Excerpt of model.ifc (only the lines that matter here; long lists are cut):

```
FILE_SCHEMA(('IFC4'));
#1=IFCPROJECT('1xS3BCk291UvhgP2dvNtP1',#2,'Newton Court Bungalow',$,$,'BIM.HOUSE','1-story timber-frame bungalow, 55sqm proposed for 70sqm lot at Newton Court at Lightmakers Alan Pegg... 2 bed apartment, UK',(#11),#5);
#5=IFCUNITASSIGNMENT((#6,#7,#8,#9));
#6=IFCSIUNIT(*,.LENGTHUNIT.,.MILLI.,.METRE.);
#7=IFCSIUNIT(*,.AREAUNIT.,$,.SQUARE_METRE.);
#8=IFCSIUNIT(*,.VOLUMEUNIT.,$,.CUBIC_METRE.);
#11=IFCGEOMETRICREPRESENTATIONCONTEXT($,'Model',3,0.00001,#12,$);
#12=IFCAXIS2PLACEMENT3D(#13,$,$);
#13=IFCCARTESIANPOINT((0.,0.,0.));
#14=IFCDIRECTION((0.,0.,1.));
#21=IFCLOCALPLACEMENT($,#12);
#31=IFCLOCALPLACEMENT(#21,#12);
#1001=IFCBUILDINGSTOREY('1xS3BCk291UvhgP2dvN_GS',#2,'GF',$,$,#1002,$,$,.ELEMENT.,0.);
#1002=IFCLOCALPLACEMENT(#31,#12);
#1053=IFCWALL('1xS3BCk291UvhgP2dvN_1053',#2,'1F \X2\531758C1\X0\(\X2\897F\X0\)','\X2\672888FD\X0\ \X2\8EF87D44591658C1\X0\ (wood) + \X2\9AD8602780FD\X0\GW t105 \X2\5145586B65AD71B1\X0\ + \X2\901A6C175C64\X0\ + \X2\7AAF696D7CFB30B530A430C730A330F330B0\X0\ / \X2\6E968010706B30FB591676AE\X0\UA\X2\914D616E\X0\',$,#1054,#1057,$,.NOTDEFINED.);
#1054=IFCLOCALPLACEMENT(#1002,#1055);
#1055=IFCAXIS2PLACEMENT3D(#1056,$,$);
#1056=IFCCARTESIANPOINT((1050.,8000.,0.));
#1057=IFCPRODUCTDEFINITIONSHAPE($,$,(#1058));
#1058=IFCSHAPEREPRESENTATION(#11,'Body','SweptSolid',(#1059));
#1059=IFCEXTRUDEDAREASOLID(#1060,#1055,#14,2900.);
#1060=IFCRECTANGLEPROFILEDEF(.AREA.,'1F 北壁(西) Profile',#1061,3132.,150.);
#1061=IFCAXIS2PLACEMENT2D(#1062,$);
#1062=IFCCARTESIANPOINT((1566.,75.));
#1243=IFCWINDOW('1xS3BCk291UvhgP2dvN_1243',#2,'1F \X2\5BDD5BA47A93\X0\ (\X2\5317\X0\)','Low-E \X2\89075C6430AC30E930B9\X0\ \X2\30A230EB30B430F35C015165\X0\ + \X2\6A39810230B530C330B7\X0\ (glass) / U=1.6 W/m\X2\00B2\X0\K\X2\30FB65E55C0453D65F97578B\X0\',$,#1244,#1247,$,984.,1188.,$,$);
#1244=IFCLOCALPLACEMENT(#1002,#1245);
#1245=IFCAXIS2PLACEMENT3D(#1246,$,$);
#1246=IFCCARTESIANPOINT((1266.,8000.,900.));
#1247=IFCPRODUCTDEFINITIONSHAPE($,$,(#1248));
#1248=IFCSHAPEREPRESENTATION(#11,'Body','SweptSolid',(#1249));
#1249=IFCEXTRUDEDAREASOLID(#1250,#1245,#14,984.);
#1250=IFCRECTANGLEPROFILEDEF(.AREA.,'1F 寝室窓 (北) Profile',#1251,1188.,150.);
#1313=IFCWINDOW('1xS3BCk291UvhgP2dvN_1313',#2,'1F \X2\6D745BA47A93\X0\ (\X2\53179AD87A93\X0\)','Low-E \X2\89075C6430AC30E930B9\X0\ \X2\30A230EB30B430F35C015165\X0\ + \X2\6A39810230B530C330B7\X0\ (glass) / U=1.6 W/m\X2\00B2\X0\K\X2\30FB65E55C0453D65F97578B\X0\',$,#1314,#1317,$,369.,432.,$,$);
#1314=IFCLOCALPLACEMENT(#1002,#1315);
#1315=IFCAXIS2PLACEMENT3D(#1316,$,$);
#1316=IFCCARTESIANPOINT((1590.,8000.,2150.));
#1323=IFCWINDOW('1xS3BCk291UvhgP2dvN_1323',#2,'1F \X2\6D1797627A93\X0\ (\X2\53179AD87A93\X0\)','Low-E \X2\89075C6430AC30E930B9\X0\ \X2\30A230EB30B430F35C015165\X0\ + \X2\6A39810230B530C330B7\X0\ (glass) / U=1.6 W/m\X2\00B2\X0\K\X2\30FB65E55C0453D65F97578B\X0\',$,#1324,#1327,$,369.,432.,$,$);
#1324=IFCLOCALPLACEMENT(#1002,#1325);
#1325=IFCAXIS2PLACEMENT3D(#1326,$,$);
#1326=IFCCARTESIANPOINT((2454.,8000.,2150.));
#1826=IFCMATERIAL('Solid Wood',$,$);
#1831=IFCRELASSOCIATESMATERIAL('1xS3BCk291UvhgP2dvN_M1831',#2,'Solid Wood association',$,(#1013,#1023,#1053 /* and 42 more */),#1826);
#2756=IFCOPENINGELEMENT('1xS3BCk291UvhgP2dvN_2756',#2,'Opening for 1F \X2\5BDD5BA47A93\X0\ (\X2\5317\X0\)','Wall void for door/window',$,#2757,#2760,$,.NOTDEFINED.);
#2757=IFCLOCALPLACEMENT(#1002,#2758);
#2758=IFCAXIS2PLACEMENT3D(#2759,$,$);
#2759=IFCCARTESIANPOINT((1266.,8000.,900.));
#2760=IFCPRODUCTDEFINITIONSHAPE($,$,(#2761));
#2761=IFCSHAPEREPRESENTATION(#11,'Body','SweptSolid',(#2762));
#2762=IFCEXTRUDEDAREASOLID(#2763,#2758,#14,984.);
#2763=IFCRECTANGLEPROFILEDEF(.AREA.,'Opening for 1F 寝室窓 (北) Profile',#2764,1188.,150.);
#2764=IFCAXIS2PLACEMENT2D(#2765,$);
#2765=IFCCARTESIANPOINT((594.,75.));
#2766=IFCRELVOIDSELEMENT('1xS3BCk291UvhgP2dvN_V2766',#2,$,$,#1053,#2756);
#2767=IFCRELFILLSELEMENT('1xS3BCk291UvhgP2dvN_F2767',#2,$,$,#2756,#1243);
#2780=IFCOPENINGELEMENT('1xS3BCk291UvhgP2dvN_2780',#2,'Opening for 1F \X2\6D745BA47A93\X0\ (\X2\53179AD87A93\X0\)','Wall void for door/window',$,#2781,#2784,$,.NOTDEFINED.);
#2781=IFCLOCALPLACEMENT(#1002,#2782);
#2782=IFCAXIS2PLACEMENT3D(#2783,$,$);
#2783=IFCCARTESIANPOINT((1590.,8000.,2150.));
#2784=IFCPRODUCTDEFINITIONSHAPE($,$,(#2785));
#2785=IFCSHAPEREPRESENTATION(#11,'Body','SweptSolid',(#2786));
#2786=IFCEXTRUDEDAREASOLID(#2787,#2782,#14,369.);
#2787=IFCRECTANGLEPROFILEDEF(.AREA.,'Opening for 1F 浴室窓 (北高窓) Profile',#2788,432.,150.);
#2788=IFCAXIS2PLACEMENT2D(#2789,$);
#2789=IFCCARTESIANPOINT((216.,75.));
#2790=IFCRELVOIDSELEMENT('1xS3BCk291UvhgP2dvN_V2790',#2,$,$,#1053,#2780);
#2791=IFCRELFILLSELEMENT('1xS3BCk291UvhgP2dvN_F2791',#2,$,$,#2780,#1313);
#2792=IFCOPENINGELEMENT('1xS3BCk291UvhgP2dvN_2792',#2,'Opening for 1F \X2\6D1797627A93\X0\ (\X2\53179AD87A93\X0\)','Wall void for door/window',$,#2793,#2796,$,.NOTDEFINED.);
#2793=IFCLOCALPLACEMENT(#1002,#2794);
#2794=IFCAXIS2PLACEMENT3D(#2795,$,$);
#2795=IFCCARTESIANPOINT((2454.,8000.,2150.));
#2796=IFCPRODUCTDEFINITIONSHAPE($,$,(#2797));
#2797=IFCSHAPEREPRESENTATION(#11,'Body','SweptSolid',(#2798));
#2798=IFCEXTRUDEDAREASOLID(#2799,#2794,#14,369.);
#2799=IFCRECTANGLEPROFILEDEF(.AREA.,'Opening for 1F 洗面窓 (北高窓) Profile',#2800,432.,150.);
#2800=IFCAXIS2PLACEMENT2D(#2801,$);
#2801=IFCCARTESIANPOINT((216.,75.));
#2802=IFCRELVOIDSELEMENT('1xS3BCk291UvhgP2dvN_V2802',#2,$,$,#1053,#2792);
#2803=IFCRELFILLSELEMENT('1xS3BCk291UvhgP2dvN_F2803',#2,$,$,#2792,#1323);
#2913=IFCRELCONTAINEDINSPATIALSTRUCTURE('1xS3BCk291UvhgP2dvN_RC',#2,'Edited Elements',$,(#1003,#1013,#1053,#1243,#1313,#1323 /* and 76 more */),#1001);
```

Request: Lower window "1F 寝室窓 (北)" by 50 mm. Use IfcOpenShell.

```python
import numpy as np
import ifcopenshell
import ifcopenshell.api.geometry
import ifcopenshell.util.placement
import ifcopenshell.util.unit

model = ifcopenshell.open("model.ifc")
unit_scale = ifcopenshell.util.unit.calculate_unit_scale(model)

window = model.by_id(1243)
opening = window.FillsVoids[0].RelatingOpeningElement
dz = -50.0

shift = np.array([0.0, 0.0, dz])
# The window is not placed relative to its opening, so move both.
for product in (opening, window):
    matrix = ifcopenshell.util.placement.get_local_placement(product.ObjectPlacement)
    matrix[:3, 3] += shift
    ifcopenshell.api.geometry.edit_object_placement(model, product=product, matrix=matrix, is_si=False)

print(f"moved by {dz * unit_scale:+.3f} m")

model.write("model_edited.ifc")
```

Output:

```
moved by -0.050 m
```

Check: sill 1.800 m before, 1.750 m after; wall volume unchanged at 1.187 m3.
